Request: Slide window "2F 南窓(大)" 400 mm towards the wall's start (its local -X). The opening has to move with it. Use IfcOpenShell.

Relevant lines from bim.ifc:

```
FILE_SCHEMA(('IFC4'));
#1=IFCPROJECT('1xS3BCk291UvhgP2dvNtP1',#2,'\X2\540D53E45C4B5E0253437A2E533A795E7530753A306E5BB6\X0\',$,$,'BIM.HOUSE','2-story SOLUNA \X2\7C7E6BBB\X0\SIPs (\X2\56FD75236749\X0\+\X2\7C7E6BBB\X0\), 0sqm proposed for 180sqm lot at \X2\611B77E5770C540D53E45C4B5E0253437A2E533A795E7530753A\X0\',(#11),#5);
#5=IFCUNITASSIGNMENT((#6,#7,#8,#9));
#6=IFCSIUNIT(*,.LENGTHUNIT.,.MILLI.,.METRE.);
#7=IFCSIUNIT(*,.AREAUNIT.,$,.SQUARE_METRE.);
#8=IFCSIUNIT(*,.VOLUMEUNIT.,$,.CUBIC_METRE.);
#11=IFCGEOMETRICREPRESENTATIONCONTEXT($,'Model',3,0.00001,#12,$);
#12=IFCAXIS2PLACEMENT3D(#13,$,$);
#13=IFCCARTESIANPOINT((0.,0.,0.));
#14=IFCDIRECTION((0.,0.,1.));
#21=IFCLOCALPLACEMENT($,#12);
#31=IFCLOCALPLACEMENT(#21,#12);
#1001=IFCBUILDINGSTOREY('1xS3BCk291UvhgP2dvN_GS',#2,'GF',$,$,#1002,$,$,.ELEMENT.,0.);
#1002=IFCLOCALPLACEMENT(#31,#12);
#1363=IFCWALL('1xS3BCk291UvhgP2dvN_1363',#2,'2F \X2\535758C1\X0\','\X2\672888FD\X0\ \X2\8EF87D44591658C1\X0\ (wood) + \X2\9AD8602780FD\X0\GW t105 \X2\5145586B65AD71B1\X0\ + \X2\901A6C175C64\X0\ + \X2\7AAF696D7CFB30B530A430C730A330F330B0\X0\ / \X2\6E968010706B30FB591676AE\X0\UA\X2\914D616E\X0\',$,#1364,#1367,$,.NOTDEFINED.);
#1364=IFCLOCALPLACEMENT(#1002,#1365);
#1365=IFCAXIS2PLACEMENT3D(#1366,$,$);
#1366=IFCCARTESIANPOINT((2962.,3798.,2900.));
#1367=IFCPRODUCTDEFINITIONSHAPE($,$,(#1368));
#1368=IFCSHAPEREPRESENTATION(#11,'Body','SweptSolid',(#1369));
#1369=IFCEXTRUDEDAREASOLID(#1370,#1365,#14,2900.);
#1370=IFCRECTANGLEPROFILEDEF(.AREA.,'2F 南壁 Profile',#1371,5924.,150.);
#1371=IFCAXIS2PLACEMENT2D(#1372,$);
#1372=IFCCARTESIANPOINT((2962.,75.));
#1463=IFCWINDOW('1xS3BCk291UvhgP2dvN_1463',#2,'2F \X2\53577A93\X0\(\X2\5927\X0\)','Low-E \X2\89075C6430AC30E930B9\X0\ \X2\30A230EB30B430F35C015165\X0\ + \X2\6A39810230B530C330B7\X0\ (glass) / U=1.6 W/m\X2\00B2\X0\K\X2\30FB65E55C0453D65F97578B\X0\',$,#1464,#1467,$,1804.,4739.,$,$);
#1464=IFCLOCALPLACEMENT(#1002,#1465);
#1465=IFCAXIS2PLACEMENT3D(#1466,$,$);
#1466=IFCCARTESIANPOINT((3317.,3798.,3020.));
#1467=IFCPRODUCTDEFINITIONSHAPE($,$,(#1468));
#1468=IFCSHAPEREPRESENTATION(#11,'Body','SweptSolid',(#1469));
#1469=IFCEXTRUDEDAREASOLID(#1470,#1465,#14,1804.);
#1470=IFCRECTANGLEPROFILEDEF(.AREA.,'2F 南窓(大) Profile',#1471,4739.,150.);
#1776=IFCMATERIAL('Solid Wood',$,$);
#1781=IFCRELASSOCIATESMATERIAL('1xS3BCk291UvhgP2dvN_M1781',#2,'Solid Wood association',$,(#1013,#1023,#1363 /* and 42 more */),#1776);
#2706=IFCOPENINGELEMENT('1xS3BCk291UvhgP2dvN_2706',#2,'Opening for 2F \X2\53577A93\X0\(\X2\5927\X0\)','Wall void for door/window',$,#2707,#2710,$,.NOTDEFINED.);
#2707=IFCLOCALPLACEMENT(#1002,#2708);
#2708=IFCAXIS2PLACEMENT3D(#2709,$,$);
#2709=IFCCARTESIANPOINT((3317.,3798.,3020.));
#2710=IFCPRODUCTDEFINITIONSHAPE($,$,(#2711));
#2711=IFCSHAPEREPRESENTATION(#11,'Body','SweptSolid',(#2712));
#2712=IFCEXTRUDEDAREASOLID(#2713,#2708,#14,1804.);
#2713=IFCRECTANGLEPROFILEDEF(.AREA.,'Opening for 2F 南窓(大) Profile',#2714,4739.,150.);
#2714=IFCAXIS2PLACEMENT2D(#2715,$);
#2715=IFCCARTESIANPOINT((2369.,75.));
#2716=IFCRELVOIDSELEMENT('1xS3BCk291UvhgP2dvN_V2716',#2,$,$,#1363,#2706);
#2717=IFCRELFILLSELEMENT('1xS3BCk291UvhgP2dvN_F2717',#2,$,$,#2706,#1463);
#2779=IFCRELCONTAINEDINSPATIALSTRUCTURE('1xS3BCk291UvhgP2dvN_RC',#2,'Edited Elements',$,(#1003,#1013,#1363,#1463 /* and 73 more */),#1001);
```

```python
import ifcopenshell
import ifcopenshell.api.geometry
import ifcopenshell.util.placement
import ifcopenshell.util.unit

model = ifcopenshell.open("bim.ifc")
unit_scale = ifcopenshell.util.unit.calculate_unit_scale(model)

window = model.by_guid("1xS3BCk291UvhgP2dvN_1463")
opening = window.FillsVoids[0].RelatingOpeningElement
wall = opening.VoidsElements[0].RelatingBuildingElement

wall_matrix = ifcopenshell.util.placement.get_local_placement(wall.ObjectPlacement)
shift = wall_matrix[:3, 0] * -0.4 / unit_scale
before = ifcopenshell.util.placement.get_local_placement(window.ObjectPlacement)[:3, 3].copy()

# The window is not placed relative to its opening, so move both.
for product in (opening, window):
    matrix = ifcopenshell.util.placement.get_local_placement(product.ObjectPlacement)
    matrix[:3, 3] += shift
    ifcopenshell.api.geometry.edit_object_placement(model, product=product, matrix=matrix, is_si=False)

after = ifcopenshell.util.placement.get_local_placement(window.ObjectPlacement)[:3, 3]
print("window moved by", (after - before).round(3) + 0.0)

model.write("bim_updated.ifc")
```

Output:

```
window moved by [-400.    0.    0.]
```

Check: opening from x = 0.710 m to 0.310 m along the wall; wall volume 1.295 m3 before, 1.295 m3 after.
